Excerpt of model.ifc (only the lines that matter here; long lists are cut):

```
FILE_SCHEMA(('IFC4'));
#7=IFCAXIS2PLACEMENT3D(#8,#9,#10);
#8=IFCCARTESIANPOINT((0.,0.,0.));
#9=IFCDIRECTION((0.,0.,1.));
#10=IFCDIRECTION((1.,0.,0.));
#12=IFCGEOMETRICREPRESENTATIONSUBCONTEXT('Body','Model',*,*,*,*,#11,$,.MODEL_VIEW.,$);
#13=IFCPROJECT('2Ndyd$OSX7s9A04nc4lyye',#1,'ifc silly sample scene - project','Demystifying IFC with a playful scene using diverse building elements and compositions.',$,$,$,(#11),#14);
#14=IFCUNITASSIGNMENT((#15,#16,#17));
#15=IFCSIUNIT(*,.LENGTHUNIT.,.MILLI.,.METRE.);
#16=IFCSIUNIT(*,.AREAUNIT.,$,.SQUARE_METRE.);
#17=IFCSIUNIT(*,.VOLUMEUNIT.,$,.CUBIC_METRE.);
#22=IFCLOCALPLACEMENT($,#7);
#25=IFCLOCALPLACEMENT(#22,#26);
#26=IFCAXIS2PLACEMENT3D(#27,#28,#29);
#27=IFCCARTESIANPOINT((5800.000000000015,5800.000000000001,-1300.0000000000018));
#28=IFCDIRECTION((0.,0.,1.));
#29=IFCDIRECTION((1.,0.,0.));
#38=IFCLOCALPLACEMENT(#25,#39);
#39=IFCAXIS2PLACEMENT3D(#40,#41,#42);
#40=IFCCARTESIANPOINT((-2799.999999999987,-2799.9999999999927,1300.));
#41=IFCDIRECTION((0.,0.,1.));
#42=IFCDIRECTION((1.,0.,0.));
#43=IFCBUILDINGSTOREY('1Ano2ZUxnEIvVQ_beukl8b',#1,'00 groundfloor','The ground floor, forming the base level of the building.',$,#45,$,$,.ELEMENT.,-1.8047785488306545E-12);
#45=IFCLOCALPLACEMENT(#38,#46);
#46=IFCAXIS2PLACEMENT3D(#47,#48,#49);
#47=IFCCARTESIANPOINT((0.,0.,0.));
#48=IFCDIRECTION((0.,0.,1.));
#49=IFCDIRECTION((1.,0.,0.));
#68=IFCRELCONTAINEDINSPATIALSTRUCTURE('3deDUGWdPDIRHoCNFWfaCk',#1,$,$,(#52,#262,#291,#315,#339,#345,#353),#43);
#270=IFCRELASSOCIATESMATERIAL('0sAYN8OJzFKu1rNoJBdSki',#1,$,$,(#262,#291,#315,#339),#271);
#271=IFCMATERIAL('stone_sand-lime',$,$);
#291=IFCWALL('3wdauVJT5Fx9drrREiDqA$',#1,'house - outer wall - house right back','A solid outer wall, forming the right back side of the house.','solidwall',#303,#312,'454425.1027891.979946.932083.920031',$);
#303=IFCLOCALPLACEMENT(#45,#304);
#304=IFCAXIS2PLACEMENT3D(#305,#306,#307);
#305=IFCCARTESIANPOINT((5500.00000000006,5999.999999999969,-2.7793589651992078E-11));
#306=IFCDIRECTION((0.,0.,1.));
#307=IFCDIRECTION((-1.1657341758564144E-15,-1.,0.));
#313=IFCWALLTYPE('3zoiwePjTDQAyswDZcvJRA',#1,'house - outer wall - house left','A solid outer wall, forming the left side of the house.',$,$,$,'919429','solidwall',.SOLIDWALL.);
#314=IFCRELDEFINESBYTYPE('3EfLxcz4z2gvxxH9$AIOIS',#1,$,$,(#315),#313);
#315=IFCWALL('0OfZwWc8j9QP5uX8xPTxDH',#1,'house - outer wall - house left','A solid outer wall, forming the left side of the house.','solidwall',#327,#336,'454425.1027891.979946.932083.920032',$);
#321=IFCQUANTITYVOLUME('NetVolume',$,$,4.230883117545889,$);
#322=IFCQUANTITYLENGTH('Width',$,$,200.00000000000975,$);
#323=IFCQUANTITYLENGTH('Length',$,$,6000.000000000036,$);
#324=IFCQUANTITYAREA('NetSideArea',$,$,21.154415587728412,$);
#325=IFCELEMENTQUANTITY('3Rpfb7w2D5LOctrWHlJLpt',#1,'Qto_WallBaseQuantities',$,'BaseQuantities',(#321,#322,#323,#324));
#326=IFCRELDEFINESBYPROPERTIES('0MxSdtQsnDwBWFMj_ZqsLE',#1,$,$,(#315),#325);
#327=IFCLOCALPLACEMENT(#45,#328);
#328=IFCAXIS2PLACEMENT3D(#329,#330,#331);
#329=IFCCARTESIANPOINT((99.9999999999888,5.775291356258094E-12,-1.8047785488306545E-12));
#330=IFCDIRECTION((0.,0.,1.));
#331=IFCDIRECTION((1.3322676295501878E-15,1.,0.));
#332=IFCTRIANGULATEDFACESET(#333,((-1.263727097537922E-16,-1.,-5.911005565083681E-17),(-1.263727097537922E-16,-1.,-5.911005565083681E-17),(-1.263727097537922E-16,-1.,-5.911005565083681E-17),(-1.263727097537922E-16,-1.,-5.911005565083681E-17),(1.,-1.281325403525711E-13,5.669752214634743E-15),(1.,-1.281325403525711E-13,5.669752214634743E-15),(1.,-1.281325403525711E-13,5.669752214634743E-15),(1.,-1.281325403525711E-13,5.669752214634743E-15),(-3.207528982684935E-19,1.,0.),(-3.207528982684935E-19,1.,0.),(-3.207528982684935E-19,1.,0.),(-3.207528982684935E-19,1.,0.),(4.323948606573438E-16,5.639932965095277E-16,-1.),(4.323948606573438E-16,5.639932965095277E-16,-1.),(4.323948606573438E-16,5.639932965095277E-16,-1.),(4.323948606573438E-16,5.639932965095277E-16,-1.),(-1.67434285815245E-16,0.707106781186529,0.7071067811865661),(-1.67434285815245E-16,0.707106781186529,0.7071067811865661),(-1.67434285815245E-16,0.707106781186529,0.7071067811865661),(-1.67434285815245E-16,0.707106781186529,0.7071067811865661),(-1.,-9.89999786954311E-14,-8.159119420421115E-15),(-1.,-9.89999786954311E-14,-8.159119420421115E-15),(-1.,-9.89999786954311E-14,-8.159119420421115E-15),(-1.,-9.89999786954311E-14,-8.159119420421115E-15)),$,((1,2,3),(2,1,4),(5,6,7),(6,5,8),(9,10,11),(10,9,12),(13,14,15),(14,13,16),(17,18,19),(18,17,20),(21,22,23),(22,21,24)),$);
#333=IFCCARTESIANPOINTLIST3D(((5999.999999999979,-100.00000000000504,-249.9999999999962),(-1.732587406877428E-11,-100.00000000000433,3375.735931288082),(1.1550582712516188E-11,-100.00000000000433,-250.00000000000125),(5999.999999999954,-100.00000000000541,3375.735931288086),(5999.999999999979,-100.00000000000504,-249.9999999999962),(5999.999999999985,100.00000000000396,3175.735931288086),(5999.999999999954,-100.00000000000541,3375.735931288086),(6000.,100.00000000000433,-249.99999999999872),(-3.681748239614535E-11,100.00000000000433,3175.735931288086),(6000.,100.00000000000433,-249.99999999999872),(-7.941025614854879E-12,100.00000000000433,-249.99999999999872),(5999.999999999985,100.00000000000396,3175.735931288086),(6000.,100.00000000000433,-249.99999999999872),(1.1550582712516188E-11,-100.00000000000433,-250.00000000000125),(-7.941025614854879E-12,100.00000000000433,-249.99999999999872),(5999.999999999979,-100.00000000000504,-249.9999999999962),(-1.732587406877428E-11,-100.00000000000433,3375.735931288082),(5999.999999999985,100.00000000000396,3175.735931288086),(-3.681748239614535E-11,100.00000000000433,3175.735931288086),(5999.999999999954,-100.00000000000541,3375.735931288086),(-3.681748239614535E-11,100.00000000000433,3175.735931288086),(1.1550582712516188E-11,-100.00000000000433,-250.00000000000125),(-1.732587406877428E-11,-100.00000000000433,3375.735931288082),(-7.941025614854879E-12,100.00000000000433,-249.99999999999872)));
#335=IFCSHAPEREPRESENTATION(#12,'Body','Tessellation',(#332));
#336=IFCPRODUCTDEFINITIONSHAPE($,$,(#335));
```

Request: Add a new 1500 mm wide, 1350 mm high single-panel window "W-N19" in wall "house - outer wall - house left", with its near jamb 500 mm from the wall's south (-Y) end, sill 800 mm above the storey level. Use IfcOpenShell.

```python
import numpy as np
import ifcopenshell
import ifcopenshell.api.feature
import ifcopenshell.api.geometry
import ifcopenshell.api.pset
import ifcopenshell.api.root
import ifcopenshell.api.spatial
import ifcopenshell.geom
import ifcopenshell.util.element
import ifcopenshell.util.placement
import ifcopenshell.util.representation
import ifcopenshell.util.shape
import ifcopenshell.util.unit

model = ifcopenshell.open("model.ifc")
unit_scale = ifcopenshell.util.unit.calculate_unit_scale(model)
area_scale = ifcopenshell.util.unit.calculate_unit_scale(model, "AREAUNIT")
volume_scale = ifcopenshell.util.unit.calculate_unit_scale(model, "VOLUMEUNIT")
settings = ifcopenshell.geom.settings()


def volume(element):
    """Net volume in cubic metres, openings subtracted."""
    shape = ifcopenshell.geom.create_shape(settings, element)
    return ifcopenshell.util.shape.get_volume(shape.geometry)


wall = model.by_guid("0OfZwWc8j9QP5uX8xPTxDH")
storey = ifcopenshell.util.element.get_container(wall, ifc_class="IfcBuildingStorey")
context = ifcopenshell.util.representation.get_context(model, "Model", "Body", "MODEL_VIEW")
before = volume(wall)

width, height, from_end, sill = 1.5, 1.35, 0.5, 0.8  # metres

# The wall runs along its own X axis, and the end named is its -X end.
wall_shape = ifcopenshell.geom.create_shape(settings, wall)
x, y, z = ifcopenshell.util.shape.get_vertices(wall_shape.geometry).T
start = x.min() + from_end
face, thickness = float(y.min()), float(y.max() - y.min())
wall_matrix = ifcopenshell.util.placement.get_local_placement(wall.ObjectPlacement)
level = ifcopenshell.util.placement.get_local_placement(storey.ObjectPlacement)[2, 3]


def in_wall(x, y):
    """Placement at x, y metres in the wall's axes, at sill height."""
    matrix = wall_matrix.copy()
    matrix[:, 3] = wall_matrix @ np.array([x / unit_scale, y / unit_scale, 0.0, 1.0])
    matrix[2, 3] = level + sill / unit_scale
    return matrix


# Opening: a box that overshoots both wall faces by 50 mm.
opening = ifcopenshell.api.root.create_entity(model, ifc_class="IfcOpeningElement", predefined_type="OPENING")
box = ifcopenshell.api.geometry.add_wall_representation(
    model, context=context, length=width, height=height, thickness=thickness + 0.1
)
ifcopenshell.api.geometry.assign_representation(model, product=opening, representation=box)
ifcopenshell.api.geometry.edit_object_placement(model, product=opening, matrix=in_wall(start, face - 0.05), is_si=False)
ifcopenshell.api.feature.add_feature(model, feature=opening, element=wall)

window = ifcopenshell.api.root.create_entity(model, ifc_class="IfcWindow", name="W-N19", predefined_type="WINDOW")
window.OverallWidth, window.OverallHeight = width / unit_scale, height / unit_scale
window.PartitioningType = "SINGLE_PANEL"
body = ifcopenshell.api.geometry.add_window_representation(
    model,
    context=context,
    overall_width=window.OverallWidth,
    overall_height=window.OverallHeight,
    partition_type="SINGLE_PANEL",
)
ifcopenshell.api.geometry.assign_representation(model, product=window, representation=body)
ifcopenshell.api.spatial.assign_container(model, products=[window], relating_structure=storey)
ifcopenshell.api.feature.add_filling(model, opening=opening, element=window)

# Centre the window in the wall's thickness.
ifcopenshell.api.geometry.edit_object_placement(model, product=window, matrix=in_wall(start, face), is_si=False)
window_shape = ifcopenshell.geom.create_shape(settings, window)
depth = ifcopenshell.util.shape.get_vertices(window_shape.geometry)[:, 1]
offset = face + thickness / 2 - (depth.min() + depth.max()) / 2
ifcopenshell.api.geometry.edit_object_placement(model, product=window, matrix=in_wall(start, offset), is_si=False)

after = volume(wall)

# Update the wall's stored quantities.
qto = model.by_id(ifcopenshell.util.element.get_pset(wall, "Qto_WallBaseQuantities", should_inherit=False)["id"])
ifcopenshell.api.pset.edit_qto(model, qto=qto, properties={
    "NetVolume": after / volume_scale,
    "NetSideArea": after / thickness / area_scale,
})

print(f"wall volume {before:.3f} -> {after:.3f} m3")

model.write("model_rev.ifc")
```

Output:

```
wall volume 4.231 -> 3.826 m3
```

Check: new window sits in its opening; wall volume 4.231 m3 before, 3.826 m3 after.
